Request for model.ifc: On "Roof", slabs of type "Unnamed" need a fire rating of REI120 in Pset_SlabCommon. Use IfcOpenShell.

First a look at what the model holds.

```python
import ifcopenshell
import ifcopenshell.util.element

model = ifcopenshell.open("model.ifc")
print(model.schema)
storey = next(s for s in model.by_type("IfcBuildingStorey") if s.Name == "Roof")
slabs = [e for e in ifcopenshell.util.element.get_decomposition(storey) if e.is_a("IfcSlab")]
seen = {}
for e in slabs:
    element_type = ifcopenshell.util.element.get_type(e)
    key = (element_type.Name if element_type != e and element_type else None, ifcopenshell.util.element.get_pset(e, "Pset_SlabCommon", "FireRating"))
    seen[key] = seen.get(key, 0) + 1
for (name, value), count in sorted(seen.items(), key=str):
    print(count, "x", name, "|", value)
```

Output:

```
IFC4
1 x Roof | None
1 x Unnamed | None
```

```python
import ifcopenshell
import ifcopenshell.api.pset
import ifcopenshell.util.element

model = ifcopenshell.open("model.ifc")

storey = next(s for s in model.by_type("IfcBuildingStorey") if s.Name == "Roof")
slabs = [e for e in ifcopenshell.util.element.get_decomposition(storey) if e.is_a("IfcSlab")]

count = 0
for e in slabs:
    element_type = ifcopenshell.util.element.get_type(e)
    if element_type in (None, e) or element_type.Name != "Unnamed":
        continue
    # add_pset returns the element's existing set when there is one.
    pset = ifcopenshell.api.pset.add_pset(model, product=e, name="Pset_SlabCommon")
    ifcopenshell.api.pset.edit_pset(model, pset=pset, properties={"FireRating": "REI120"})
    count += 1

print(count, "slabs updated")

model.write("model_edited.ifc")
```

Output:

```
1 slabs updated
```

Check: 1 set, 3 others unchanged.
